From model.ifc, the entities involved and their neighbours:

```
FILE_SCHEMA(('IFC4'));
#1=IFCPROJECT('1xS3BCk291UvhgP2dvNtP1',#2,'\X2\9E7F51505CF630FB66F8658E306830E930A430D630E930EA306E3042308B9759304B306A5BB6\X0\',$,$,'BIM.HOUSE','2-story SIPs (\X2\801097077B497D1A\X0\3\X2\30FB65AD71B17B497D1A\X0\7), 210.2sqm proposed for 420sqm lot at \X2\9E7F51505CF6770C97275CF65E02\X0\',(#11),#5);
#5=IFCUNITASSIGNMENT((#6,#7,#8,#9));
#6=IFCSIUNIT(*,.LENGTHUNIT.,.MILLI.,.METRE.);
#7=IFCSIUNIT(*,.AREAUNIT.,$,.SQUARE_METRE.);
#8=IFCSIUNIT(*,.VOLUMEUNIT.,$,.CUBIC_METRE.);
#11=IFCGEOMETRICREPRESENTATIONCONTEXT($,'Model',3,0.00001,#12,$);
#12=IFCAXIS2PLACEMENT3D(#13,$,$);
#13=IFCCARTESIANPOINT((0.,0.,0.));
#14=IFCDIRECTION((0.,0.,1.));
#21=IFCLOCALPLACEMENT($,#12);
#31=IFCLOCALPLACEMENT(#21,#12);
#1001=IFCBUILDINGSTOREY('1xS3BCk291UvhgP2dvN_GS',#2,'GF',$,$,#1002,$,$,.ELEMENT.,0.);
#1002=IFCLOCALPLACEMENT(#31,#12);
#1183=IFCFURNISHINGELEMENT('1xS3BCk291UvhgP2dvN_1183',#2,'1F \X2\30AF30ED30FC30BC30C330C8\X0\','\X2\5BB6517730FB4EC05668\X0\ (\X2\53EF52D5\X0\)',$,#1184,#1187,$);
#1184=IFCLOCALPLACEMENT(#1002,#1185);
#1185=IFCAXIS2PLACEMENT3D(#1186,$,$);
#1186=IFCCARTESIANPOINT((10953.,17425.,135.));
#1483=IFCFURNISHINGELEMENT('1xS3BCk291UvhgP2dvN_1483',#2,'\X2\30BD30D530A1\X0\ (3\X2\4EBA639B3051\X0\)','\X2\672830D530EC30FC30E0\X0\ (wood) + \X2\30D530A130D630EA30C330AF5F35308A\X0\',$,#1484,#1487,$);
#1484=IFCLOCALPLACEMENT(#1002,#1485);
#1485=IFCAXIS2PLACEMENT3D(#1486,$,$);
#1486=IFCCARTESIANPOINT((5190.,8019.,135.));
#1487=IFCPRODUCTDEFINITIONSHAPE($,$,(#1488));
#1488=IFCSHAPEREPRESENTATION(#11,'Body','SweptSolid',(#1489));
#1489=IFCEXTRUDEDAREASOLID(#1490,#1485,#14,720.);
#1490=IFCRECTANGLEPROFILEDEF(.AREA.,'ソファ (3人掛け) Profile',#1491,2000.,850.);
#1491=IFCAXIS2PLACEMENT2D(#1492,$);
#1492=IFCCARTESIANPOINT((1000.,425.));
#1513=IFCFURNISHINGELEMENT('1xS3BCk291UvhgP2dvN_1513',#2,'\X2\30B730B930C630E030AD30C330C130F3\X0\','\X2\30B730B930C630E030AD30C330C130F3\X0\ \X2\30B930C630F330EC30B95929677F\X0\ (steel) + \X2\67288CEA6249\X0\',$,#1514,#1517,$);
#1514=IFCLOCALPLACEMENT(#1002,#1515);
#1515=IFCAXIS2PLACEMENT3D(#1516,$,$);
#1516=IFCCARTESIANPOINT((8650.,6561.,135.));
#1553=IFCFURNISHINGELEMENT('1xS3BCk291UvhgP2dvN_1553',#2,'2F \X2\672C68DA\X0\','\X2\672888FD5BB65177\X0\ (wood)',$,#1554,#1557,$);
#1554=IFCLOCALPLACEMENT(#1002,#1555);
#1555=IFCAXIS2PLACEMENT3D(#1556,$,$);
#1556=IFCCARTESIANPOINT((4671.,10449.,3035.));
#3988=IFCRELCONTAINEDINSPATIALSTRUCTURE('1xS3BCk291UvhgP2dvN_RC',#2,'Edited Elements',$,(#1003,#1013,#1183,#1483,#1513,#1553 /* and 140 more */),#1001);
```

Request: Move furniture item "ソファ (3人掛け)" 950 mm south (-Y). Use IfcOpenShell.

```python
import ifcopenshell
import ifcopenshell.api.geometry
import ifcopenshell.util.placement
import ifcopenshell.util.unit

model = ifcopenshell.open("model.ifc")
unit_scale = ifcopenshell.util.unit.calculate_unit_scale(model)

item = model.by_guid("1xS3BCk291UvhgP2dvN_1483")
matrix = ifcopenshell.util.placement.get_local_placement(item.ObjectPlacement)
matrix[1, 3] -= 0.95 / unit_scale
ifcopenshell.api.geometry.edit_object_placement(model, product=item, matrix=matrix, is_si=False)

print(ifcopenshell.util.placement.get_local_placement(item.ObjectPlacement).round(3) + 0.0)

model.write("model_v2.ifc")
```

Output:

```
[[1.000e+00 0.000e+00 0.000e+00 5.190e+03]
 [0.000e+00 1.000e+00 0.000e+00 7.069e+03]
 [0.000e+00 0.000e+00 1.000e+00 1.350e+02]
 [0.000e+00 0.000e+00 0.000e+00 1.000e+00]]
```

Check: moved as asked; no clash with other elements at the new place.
